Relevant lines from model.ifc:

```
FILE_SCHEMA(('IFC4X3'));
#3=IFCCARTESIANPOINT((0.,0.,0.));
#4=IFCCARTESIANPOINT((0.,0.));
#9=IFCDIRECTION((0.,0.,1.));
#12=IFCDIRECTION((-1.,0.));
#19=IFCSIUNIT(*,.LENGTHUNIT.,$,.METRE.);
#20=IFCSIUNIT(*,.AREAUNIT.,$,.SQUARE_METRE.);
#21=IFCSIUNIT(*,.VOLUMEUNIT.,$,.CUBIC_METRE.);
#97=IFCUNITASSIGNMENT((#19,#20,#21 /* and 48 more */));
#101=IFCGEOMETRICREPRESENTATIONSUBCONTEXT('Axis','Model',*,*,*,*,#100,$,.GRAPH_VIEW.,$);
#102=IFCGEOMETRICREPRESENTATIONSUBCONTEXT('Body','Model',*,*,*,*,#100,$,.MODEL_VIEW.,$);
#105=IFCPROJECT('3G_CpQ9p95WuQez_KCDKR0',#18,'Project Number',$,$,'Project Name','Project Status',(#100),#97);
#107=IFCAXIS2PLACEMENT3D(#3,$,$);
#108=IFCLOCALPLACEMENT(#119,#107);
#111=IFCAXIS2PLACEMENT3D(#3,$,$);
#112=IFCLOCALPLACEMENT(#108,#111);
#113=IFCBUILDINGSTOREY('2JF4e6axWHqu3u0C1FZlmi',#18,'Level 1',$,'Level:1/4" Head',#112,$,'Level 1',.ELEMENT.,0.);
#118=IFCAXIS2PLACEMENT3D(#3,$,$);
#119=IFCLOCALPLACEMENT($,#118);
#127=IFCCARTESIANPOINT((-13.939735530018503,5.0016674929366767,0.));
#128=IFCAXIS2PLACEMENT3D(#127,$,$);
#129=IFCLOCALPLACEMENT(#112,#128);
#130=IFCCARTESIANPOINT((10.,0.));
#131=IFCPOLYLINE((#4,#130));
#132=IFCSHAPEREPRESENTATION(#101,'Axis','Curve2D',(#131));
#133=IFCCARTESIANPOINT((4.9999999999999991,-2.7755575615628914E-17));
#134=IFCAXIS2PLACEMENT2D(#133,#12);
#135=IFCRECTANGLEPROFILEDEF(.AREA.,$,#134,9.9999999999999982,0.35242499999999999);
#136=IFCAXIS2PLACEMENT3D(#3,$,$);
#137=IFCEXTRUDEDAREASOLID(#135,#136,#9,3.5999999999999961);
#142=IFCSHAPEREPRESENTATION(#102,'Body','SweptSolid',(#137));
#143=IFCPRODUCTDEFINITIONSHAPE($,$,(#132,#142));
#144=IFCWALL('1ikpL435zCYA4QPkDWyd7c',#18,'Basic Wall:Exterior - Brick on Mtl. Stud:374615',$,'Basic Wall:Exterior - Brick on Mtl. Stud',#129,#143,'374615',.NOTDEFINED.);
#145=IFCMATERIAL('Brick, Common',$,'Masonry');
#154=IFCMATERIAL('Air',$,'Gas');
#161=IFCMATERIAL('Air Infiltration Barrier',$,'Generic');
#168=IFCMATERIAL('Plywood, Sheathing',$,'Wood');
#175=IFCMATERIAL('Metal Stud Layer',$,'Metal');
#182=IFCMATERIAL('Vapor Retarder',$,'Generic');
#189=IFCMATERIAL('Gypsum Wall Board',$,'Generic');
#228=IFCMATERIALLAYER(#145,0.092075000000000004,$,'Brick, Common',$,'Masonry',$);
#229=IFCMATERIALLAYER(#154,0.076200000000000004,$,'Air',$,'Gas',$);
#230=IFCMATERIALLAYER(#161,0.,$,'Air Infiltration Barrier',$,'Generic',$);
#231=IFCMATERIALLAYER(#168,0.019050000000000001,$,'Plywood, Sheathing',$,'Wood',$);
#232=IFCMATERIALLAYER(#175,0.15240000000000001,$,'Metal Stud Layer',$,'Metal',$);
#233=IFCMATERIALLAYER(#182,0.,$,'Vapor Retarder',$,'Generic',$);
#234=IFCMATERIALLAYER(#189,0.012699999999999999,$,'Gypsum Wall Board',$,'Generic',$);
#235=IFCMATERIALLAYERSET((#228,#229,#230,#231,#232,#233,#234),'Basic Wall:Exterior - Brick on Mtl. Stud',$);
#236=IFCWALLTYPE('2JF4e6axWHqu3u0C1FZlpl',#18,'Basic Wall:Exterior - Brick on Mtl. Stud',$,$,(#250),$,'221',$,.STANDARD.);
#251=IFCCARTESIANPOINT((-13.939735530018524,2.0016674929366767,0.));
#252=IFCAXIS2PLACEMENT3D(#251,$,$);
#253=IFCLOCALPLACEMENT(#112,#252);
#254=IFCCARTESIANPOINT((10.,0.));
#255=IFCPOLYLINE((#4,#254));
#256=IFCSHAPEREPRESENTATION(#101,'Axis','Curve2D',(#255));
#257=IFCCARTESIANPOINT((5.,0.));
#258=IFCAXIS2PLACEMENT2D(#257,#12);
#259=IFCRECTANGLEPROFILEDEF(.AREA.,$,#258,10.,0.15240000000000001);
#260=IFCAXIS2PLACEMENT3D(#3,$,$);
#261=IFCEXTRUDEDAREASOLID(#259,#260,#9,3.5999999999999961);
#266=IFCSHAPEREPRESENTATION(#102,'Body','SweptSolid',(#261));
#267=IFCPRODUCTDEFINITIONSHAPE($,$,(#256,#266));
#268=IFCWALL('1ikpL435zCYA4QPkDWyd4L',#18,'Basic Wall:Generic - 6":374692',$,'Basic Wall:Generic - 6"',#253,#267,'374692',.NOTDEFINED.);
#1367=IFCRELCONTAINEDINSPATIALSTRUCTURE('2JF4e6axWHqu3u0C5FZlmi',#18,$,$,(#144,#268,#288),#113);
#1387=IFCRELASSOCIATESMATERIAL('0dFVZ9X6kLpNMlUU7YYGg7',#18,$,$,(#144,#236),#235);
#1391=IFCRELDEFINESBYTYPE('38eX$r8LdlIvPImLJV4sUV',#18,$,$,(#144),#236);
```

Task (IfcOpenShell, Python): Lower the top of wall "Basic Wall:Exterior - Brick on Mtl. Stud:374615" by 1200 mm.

```python
import ifcopenshell
import ifcopenshell.geom
import ifcopenshell.util.representation
import ifcopenshell.util.shape
import ifcopenshell.util.unit

model = ifcopenshell.open("model.ifc")
unit_scale = ifcopenshell.util.unit.calculate_unit_scale(model)
settings = ifcopenshell.geom.settings()


def volume(element):
    """Net volume in cubic metres, openings subtracted."""
    shape = ifcopenshell.geom.create_shape(settings, element)
    return ifcopenshell.util.shape.get_volume(shape.geometry)


wall = model.by_guid("1ikpL435zCYA4QPkDWyd7c")
before = volume(wall)

body = ifcopenshell.util.representation.get_representation(wall, "Model", "Body")
solid = body.Items[0]
old_height = solid.Depth
solid.Depth -= 1.2 / unit_scale
after = volume(wall)

print(f"height {old_height:g} -> {solid.Depth:g}, volume {before:.3f} -> {after:.3f} m3")

model.write("model_edited.ifc")
```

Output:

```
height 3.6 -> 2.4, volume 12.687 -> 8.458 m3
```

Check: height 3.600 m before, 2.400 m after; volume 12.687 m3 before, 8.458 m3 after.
